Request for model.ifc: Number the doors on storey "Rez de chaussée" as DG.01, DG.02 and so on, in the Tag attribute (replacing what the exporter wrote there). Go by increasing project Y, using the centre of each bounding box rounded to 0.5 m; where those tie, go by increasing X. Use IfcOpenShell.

First a look at what the model holds.

```python
import ifcopenshell
import ifcopenshell.util.element
import ifcopenshell.util.placement

model = ifcopenshell.open("model.ifc")
print(model.schema)
storey = next(s for s in model.by_type("IfcBuildingStorey") if s.Name == "Rez de chaussée")
doors = [e for e in ifcopenshell.util.element.get_decomposition(storey) if e.is_a("IfcDoor")]
for e in sorted(doors, key=lambda e: e.id()):
    origin = ifcopenshell.util.placement.get_local_placement(e.ObjectPlacement)[:3, 3]
    print(e.id(), e.Tag, e.Name, origin.round(2) + 0.0, sep=" | ")
```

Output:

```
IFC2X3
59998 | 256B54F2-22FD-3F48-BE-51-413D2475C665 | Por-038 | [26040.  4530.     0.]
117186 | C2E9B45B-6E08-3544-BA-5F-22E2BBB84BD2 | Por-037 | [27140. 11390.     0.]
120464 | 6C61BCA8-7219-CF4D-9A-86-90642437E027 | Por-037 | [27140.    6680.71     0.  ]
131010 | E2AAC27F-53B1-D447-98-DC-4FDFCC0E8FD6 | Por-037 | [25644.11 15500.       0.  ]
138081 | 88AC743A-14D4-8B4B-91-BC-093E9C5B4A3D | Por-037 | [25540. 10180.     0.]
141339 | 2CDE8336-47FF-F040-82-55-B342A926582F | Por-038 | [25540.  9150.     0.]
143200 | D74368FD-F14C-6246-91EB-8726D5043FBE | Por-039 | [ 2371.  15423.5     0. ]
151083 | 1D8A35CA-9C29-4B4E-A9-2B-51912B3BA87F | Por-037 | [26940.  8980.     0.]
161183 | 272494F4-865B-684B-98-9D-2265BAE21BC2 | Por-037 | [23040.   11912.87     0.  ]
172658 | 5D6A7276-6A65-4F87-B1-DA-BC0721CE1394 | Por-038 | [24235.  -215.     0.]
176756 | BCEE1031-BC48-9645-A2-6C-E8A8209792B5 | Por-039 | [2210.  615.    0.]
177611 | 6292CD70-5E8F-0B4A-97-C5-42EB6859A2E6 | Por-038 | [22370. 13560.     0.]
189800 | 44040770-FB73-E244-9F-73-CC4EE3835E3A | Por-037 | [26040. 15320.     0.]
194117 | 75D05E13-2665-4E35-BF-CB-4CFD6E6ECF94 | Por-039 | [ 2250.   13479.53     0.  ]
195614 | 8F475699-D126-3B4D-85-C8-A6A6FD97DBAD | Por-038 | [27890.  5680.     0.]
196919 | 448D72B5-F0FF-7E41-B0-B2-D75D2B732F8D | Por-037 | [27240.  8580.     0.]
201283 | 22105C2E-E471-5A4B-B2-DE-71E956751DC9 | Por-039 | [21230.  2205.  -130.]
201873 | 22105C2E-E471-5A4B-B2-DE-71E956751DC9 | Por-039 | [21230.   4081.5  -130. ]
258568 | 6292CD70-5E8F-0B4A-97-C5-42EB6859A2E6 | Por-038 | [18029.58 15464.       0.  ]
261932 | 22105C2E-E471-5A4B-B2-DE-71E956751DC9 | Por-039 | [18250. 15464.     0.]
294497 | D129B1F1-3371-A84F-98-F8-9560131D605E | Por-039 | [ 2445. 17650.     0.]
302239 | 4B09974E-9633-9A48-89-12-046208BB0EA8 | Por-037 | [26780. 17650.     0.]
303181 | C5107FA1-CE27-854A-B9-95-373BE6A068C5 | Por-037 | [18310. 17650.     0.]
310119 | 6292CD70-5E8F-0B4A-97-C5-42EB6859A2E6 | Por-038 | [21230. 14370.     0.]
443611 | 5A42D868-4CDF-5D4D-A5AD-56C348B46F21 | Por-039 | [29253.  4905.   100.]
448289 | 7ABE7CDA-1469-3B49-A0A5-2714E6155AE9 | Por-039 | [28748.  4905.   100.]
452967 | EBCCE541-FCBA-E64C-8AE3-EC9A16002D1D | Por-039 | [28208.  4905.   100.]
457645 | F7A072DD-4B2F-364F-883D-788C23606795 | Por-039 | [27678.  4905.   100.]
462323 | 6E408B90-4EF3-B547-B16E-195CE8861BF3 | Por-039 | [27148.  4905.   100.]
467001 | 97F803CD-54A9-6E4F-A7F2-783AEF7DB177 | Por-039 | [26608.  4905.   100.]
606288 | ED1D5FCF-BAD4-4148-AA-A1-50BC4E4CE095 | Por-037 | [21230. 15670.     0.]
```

```python
import ifcopenshell
import ifcopenshell.geom
import ifcopenshell.util.element
import ifcopenshell.util.shape

model = ifcopenshell.open("model.ifc")
settings = ifcopenshell.geom.settings()
settings.set("use-world-coords", True)


def centre(element):
    shape = ifcopenshell.geom.create_shape(settings, element)
    return ifcopenshell.util.shape.get_bbox_centroid(shape.geometry)


storey = next(s for s in model.by_type("IfcBuildingStorey") if s.Name == "Rez de chaussée")
doors = [e for e in ifcopenshell.util.element.get_decomposition(storey) if e.is_a("IfcDoor")]

# Insertion points can sit at a corner or the storey origin, so sort by the geometry (in metres).
centres = {e: centre(e) for e in doors}
doors.sort(key=lambda e: (round(centres[e][1] / 0.5), centres[e][0]))

for i, e in enumerate(doors, start=1):
    number = f"DG.{i:02d}"
    e.Tag = number
    print(e.id(), number)

model.write("model-out.ifc")
```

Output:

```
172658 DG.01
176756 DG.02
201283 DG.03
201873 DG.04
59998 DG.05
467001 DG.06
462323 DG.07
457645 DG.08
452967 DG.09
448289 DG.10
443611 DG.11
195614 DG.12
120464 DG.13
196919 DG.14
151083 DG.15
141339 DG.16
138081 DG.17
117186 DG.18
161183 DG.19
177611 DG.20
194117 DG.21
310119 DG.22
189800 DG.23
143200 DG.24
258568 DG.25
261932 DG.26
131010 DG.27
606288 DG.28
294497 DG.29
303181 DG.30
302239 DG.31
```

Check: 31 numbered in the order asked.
